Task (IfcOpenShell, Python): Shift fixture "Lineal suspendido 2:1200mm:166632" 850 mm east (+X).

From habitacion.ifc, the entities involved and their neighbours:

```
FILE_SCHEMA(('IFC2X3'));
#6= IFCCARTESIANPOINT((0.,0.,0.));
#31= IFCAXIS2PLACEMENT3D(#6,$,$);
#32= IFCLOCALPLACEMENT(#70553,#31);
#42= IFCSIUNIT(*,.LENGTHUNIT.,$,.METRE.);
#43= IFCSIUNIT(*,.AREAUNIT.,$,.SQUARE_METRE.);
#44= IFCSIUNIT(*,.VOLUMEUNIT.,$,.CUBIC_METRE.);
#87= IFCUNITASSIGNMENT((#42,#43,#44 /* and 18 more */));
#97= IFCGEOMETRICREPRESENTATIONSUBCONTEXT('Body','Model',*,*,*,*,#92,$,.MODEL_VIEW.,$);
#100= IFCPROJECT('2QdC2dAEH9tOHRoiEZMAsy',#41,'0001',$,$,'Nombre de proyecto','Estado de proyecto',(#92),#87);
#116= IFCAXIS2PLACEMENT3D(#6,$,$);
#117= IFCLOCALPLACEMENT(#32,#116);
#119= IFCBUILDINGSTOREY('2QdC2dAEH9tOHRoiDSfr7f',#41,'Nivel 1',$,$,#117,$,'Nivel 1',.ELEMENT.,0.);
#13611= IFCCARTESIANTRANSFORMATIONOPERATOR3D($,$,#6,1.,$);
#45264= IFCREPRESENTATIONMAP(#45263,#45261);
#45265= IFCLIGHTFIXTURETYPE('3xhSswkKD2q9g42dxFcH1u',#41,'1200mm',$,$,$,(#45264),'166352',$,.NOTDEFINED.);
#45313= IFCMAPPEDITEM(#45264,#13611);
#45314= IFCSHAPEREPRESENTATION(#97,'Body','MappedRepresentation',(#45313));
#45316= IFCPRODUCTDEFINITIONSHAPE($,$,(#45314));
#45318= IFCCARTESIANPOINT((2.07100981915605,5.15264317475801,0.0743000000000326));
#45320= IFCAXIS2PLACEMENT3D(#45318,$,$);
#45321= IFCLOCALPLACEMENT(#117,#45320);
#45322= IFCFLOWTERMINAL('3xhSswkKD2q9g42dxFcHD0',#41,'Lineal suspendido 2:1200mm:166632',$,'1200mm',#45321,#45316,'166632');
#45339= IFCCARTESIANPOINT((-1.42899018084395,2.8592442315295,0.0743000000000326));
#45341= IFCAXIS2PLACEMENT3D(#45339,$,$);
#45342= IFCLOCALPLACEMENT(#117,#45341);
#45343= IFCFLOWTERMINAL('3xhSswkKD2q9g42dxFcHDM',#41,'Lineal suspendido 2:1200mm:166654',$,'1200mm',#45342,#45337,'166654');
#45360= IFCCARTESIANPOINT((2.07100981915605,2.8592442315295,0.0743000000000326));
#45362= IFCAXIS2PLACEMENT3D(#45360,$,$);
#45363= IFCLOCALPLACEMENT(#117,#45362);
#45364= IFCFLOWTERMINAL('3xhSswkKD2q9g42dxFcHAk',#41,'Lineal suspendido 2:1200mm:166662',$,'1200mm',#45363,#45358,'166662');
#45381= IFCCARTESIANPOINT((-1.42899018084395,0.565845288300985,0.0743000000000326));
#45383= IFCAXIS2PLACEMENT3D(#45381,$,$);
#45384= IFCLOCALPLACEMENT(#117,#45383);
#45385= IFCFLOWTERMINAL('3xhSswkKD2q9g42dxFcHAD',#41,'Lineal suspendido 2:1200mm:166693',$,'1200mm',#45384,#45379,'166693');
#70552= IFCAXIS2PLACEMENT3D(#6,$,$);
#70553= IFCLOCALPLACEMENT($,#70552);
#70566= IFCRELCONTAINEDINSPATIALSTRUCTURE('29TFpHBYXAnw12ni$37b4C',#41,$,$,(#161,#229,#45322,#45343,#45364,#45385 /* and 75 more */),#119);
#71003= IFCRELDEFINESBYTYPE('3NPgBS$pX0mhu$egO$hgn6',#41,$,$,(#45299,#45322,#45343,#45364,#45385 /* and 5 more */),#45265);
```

```python
import ifcopenshell
import ifcopenshell.api.geometry
import ifcopenshell.util.placement

model = ifcopenshell.open("habitacion.ifc")

item = model.by_guid("3xhSswkKD2q9g42dxFcHD0")
matrix = ifcopenshell.util.placement.get_local_placement(item.ObjectPlacement)
matrix[0, 3] += 0.85
ifcopenshell.api.geometry.edit_object_placement(model, product=item, matrix=matrix, is_si=False)

print(ifcopenshell.util.placement.get_local_placement(item.ObjectPlacement).round(3) + 0.0)

model.write("habitacion_edited.ifc")
```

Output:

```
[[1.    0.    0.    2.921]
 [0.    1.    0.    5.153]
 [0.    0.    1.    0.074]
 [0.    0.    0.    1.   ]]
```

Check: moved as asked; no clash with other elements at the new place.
